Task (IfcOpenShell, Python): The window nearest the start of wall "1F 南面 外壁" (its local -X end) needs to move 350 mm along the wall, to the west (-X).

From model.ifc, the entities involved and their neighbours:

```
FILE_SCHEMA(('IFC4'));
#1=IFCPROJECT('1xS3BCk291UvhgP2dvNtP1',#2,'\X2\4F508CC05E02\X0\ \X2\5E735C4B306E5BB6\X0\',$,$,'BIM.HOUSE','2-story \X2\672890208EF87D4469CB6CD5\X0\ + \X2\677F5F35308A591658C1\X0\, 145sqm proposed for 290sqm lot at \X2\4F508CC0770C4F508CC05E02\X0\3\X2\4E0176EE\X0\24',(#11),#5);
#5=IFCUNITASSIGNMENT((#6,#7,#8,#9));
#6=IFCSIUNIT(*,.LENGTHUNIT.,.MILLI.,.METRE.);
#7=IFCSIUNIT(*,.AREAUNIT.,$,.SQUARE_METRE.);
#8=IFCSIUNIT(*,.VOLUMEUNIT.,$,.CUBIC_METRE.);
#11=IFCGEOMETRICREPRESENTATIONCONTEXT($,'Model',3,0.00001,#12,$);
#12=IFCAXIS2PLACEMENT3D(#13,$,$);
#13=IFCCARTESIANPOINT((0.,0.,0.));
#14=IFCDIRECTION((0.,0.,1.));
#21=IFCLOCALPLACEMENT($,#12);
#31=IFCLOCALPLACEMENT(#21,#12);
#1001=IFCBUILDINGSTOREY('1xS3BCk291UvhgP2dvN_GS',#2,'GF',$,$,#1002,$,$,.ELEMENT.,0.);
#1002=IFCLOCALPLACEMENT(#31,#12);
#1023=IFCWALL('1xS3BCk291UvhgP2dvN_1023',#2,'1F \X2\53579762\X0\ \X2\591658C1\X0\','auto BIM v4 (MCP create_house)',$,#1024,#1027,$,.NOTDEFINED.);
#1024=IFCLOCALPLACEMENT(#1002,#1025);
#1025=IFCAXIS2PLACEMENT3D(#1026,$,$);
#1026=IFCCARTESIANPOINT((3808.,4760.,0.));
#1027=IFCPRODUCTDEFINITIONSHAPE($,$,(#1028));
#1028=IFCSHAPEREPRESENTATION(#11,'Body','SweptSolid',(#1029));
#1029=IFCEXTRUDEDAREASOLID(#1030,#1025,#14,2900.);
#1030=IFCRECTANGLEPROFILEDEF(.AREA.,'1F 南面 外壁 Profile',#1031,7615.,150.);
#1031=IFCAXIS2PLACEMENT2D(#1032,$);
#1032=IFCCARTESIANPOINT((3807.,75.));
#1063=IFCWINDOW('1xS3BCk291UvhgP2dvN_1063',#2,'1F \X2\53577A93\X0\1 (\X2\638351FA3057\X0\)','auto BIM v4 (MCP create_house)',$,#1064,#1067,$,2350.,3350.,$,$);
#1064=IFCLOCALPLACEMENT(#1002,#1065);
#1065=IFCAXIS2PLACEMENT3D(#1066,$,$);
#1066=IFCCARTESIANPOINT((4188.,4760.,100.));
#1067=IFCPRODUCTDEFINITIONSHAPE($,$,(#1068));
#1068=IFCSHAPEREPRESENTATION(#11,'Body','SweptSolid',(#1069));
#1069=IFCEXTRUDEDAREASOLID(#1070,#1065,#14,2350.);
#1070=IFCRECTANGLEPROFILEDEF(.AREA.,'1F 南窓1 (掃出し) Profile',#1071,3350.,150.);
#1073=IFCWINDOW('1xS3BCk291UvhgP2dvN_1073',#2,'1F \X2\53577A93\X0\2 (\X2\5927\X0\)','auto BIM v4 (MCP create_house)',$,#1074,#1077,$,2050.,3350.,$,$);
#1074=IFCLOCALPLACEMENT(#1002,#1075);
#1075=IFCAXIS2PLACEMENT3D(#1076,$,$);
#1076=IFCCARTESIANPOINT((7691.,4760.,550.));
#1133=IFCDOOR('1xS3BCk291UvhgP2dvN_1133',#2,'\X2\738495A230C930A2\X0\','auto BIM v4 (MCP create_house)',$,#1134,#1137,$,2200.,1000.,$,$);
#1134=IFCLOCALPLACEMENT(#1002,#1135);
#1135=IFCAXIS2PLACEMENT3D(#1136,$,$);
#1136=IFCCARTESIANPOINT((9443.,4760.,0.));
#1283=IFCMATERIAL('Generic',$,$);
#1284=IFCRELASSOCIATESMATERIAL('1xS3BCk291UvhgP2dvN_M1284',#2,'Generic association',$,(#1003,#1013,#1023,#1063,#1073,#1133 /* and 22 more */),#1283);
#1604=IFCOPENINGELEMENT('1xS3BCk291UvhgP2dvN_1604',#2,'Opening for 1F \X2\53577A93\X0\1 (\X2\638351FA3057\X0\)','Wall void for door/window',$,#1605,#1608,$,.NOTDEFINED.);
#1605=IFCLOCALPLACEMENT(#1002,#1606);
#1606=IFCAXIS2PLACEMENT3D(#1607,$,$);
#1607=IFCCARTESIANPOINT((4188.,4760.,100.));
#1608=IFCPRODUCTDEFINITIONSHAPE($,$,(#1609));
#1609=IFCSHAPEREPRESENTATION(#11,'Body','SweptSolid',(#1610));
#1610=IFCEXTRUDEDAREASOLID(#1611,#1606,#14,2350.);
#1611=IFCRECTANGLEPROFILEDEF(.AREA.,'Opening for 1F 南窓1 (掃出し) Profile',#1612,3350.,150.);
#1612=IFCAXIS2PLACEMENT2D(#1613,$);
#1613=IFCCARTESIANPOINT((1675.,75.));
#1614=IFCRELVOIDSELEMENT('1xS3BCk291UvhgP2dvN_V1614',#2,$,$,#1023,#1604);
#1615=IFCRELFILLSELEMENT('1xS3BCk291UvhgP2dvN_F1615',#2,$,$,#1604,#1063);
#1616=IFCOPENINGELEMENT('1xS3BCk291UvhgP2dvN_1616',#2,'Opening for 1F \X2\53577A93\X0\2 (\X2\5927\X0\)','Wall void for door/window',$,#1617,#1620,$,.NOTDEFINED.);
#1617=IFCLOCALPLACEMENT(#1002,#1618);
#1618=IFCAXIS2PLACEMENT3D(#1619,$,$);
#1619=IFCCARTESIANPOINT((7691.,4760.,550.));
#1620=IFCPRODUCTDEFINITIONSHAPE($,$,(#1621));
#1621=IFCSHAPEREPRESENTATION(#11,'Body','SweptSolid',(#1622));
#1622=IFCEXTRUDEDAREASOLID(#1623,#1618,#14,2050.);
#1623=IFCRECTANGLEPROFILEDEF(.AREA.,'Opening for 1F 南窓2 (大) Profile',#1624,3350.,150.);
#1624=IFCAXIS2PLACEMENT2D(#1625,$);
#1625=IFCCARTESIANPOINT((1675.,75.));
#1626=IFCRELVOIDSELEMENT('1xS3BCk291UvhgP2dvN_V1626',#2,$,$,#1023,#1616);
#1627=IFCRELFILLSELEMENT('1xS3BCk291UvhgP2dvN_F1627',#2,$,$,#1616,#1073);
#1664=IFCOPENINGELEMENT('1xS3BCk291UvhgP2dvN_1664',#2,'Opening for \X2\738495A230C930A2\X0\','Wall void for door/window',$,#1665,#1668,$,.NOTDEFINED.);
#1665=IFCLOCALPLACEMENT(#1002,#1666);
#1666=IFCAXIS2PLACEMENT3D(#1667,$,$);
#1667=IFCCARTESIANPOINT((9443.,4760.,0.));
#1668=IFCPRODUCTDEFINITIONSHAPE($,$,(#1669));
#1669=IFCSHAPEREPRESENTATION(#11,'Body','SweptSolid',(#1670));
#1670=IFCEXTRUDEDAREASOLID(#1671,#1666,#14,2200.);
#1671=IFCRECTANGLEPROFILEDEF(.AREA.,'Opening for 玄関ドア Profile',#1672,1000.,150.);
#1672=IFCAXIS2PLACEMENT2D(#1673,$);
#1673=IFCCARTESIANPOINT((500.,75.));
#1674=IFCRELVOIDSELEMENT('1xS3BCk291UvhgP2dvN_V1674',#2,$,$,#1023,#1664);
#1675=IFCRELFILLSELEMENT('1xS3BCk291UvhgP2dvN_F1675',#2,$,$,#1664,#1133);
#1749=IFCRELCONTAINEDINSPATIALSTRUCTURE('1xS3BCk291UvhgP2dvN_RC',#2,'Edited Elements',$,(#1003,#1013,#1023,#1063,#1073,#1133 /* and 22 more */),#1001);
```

```python
import ifcopenshell
import ifcopenshell.api.geometry
import ifcopenshell.util.placement

model = ifcopenshell.open("model.ifc")

window = model.by_guid("1xS3BCk291UvhgP2dvN_1063")
opening = window.FillsVoids[0].RelatingOpeningElement
wall = opening.VoidsElements[0].RelatingBuildingElement

wall_matrix = ifcopenshell.util.placement.get_local_placement(wall.ObjectPlacement)
shift = wall_matrix[:3, 0] * -350.0
before = ifcopenshell.util.placement.get_local_placement(window.ObjectPlacement)[:3, 3].copy()

# The window is not placed relative to its opening, so move both.
for product in (opening, window):
    matrix = ifcopenshell.util.placement.get_local_placement(product.ObjectPlacement)
    matrix[:3, 3] += shift
    ifcopenshell.api.geometry.edit_object_placement(model, product=product, matrix=matrix, is_si=False)

after = ifcopenshell.util.placement.get_local_placement(window.ObjectPlacement)[:3, 3]
print("window moved by", (after - before).round(3) + 0.0)

model.write("model_v2.ifc")
```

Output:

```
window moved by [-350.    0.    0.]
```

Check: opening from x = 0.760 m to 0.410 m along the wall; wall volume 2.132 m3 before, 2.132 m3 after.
